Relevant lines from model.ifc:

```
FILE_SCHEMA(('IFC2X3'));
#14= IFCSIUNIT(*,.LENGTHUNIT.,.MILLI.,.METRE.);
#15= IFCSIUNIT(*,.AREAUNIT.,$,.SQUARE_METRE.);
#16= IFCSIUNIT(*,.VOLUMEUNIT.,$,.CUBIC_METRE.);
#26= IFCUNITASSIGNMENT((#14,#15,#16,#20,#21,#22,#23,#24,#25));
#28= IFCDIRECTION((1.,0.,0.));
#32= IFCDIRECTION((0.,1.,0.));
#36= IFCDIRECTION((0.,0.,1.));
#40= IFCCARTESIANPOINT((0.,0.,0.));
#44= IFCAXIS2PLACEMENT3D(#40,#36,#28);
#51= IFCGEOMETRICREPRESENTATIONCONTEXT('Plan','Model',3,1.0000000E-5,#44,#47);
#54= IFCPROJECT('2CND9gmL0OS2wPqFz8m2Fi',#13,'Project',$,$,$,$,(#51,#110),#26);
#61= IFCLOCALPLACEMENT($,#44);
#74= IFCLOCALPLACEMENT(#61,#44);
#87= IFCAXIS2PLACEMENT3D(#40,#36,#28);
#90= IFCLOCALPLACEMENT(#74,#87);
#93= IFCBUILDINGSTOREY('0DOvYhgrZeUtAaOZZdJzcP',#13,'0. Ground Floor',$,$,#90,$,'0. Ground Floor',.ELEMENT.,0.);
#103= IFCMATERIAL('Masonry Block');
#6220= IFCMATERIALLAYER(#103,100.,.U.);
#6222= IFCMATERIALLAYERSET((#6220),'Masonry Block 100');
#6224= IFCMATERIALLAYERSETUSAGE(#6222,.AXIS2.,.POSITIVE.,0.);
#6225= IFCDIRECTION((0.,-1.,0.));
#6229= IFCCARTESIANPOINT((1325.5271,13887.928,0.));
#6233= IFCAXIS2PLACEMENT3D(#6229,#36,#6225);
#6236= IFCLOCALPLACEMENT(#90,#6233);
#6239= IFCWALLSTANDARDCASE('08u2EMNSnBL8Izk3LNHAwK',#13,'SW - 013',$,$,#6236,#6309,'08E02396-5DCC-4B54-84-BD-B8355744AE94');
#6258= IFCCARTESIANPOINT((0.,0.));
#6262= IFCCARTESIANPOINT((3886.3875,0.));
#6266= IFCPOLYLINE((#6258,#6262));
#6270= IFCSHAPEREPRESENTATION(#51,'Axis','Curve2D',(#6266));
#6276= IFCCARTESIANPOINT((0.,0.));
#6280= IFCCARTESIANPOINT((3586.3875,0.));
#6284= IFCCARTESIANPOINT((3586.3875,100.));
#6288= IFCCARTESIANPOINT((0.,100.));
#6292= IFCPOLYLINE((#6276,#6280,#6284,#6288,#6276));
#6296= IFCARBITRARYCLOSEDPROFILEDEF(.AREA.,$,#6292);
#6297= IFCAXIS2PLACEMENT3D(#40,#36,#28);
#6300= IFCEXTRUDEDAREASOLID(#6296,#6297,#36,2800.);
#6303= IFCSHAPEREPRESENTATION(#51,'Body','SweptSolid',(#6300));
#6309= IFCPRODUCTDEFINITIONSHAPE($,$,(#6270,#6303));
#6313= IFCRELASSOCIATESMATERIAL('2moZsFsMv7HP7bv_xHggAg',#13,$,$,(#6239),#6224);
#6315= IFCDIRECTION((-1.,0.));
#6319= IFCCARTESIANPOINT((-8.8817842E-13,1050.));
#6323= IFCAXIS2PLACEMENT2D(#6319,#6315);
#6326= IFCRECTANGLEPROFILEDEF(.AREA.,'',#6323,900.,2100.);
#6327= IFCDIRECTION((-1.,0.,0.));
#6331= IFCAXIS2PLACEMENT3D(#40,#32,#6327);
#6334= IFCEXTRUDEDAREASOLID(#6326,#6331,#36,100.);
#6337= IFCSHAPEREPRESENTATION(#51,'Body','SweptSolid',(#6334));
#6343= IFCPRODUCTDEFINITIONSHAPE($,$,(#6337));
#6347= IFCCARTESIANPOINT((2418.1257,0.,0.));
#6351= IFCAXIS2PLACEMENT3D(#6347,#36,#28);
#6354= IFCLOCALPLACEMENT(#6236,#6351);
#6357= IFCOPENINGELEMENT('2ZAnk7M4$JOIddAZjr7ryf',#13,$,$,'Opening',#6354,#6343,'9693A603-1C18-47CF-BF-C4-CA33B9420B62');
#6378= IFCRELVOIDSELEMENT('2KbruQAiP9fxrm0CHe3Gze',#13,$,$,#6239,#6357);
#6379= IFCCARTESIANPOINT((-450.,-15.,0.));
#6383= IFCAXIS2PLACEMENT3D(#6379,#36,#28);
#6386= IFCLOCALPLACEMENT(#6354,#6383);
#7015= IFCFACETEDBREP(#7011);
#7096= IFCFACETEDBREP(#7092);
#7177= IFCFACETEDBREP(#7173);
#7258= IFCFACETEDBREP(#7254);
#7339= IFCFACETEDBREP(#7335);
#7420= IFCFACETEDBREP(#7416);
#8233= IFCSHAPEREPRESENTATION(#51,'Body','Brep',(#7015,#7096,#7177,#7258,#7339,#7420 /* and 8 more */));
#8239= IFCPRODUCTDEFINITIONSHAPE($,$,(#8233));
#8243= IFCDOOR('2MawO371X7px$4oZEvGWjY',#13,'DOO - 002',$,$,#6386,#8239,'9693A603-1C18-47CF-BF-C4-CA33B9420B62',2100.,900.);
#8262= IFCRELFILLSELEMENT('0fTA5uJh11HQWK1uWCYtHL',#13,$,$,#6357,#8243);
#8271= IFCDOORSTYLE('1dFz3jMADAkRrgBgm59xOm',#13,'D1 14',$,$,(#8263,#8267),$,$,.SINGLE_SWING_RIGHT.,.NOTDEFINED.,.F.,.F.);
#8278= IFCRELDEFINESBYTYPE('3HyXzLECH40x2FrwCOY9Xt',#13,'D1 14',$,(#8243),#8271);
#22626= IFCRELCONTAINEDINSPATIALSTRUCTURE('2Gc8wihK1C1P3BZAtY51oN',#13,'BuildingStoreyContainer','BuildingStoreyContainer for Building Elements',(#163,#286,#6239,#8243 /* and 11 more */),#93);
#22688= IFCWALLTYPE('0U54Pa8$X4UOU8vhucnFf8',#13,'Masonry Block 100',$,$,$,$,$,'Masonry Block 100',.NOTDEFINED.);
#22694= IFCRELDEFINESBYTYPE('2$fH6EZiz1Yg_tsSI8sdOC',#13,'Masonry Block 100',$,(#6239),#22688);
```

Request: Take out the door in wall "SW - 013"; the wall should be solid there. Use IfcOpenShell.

```python
import ifcopenshell
import ifcopenshell.api.feature
import ifcopenshell.api.root
import ifcopenshell.geom
import ifcopenshell.util.shape

model = ifcopenshell.open("model.ifc")
settings = ifcopenshell.geom.settings()


def volume(element):
    """Net volume in cubic metres, openings subtracted."""
    shape = ifcopenshell.geom.create_shape(settings, element)
    return ifcopenshell.util.shape.get_volume(shape.geometry)


door = model.by_id(8243)
opening = door.FillsVoids[0].RelatingOpeningElement
wall = opening.VoidsElements[0].RelatingBuildingElement
before = volume(wall)

ifcopenshell.api.root.remove_product(model, product=door)
ifcopenshell.api.feature.remove_feature(model, feature=opening)

after = volume(wall)

print(f"wall volume {before:.3f} -> {after:.3f} m3")

model.write("model-out.ifc")
```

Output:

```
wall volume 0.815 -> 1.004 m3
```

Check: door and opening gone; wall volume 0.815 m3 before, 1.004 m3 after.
